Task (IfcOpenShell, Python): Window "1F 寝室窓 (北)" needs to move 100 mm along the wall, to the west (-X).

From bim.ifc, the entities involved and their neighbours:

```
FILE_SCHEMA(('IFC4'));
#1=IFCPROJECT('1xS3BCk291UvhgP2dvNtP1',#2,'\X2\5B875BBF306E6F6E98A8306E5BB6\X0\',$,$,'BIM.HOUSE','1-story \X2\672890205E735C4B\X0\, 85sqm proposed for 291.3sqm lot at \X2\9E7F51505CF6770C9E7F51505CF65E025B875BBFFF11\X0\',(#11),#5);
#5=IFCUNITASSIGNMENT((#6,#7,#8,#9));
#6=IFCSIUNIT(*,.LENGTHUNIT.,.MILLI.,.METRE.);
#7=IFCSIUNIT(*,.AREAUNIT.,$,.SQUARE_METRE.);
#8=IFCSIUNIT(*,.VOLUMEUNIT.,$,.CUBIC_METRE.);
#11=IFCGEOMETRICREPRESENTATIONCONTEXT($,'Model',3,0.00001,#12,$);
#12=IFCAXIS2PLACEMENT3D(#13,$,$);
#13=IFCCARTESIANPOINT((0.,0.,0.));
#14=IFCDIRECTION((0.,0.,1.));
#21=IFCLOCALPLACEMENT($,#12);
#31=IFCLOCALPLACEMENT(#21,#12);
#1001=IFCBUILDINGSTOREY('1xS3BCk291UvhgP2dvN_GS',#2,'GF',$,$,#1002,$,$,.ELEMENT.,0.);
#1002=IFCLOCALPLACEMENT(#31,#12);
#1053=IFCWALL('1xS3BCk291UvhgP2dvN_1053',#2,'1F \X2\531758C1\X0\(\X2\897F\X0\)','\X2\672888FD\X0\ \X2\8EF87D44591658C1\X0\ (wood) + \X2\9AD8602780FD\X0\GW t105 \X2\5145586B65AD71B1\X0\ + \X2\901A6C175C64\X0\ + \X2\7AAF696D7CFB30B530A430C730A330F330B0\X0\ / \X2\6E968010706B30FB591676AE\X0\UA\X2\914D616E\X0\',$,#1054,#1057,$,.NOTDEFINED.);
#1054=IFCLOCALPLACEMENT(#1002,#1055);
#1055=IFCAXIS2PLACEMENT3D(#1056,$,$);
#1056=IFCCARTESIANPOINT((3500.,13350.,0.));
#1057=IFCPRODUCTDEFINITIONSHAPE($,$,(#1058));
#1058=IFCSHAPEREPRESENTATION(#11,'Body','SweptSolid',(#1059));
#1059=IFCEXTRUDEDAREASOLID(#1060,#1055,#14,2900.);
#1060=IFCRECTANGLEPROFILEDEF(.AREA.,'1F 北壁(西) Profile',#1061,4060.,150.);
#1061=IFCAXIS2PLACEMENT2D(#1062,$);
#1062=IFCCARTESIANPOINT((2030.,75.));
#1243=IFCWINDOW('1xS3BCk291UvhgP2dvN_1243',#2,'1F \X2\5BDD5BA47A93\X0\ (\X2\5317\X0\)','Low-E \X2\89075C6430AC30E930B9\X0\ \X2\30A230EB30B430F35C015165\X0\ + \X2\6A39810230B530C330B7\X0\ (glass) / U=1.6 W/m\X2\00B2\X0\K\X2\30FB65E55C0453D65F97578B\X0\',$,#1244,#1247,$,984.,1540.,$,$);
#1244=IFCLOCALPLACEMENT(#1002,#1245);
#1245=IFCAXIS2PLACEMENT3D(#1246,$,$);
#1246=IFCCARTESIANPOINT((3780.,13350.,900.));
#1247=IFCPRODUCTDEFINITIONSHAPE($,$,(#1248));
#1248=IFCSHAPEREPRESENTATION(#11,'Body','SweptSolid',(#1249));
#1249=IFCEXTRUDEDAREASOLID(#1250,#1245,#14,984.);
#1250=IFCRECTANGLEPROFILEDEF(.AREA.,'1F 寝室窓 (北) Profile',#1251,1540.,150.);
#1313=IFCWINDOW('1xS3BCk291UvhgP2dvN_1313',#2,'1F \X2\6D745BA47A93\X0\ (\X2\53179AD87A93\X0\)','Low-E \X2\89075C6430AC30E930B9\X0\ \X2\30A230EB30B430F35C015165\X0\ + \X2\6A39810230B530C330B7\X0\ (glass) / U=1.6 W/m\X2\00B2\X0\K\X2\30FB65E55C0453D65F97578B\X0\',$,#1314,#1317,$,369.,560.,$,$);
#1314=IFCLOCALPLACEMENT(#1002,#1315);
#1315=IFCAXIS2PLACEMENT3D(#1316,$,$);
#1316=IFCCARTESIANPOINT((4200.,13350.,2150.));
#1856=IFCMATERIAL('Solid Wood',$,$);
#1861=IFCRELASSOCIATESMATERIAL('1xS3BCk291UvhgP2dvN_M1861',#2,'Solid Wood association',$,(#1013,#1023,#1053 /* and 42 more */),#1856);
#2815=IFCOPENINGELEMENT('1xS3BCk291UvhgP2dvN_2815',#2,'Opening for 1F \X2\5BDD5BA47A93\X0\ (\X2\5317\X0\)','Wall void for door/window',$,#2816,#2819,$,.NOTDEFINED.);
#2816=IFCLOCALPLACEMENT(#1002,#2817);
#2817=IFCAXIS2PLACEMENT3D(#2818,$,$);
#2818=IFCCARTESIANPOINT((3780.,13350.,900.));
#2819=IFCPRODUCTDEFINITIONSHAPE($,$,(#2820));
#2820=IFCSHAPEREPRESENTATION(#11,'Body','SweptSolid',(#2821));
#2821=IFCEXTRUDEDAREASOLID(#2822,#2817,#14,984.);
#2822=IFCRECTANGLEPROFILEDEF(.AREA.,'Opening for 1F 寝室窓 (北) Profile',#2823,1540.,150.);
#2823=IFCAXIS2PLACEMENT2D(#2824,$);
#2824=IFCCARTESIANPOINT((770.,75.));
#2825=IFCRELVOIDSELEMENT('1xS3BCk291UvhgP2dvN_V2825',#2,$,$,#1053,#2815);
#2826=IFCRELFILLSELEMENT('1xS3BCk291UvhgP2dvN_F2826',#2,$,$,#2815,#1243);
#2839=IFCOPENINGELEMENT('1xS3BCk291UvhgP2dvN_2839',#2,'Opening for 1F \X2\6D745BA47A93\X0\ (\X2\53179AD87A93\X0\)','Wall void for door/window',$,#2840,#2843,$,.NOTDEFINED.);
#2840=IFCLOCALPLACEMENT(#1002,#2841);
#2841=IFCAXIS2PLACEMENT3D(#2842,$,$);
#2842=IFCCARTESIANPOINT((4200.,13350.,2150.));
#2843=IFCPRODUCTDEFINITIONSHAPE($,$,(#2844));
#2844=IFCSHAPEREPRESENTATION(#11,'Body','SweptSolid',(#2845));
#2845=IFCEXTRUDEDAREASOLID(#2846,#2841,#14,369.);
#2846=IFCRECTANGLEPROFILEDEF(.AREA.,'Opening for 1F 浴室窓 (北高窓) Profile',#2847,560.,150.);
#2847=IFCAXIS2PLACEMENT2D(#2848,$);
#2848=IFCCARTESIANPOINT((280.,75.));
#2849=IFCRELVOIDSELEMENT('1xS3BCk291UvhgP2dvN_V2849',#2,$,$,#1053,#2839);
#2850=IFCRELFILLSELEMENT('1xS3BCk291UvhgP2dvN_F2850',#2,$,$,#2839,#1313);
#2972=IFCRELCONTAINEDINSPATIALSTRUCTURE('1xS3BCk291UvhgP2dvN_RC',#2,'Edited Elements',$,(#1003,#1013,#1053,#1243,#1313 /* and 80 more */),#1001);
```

```python
import ifcopenshell
import ifcopenshell.api.geometry
import ifcopenshell.util.placement

model = ifcopenshell.open("bim.ifc")

window = model.by_guid("1xS3BCk291UvhgP2dvN_1243")
opening = window.FillsVoids[0].RelatingOpeningElement
wall = opening.VoidsElements[0].RelatingBuildingElement

wall_matrix = ifcopenshell.util.placement.get_local_placement(wall.ObjectPlacement)
shift = wall_matrix[:3, 0] * -100.0
before = ifcopenshell.util.placement.get_local_placement(window.ObjectPlacement)[:3, 3].copy()

# The window is not placed relative to its opening, so move both.
for product in (opening, window):
    matrix = ifcopenshell.util.placement.get_local_placement(product.ObjectPlacement)
    matrix[:3, 3] += shift
    ifcopenshell.api.geometry.edit_object_placement(model, product=product, matrix=matrix, is_si=False)

after = ifcopenshell.util.placement.get_local_placement(window.ObjectPlacement)[:3, 3]
print("window moved by", (after - before).round(3) + 0.0)

model.write("bim_rev.ifc")
```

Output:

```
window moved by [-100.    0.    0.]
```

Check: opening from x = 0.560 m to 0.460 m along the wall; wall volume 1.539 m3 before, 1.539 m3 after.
